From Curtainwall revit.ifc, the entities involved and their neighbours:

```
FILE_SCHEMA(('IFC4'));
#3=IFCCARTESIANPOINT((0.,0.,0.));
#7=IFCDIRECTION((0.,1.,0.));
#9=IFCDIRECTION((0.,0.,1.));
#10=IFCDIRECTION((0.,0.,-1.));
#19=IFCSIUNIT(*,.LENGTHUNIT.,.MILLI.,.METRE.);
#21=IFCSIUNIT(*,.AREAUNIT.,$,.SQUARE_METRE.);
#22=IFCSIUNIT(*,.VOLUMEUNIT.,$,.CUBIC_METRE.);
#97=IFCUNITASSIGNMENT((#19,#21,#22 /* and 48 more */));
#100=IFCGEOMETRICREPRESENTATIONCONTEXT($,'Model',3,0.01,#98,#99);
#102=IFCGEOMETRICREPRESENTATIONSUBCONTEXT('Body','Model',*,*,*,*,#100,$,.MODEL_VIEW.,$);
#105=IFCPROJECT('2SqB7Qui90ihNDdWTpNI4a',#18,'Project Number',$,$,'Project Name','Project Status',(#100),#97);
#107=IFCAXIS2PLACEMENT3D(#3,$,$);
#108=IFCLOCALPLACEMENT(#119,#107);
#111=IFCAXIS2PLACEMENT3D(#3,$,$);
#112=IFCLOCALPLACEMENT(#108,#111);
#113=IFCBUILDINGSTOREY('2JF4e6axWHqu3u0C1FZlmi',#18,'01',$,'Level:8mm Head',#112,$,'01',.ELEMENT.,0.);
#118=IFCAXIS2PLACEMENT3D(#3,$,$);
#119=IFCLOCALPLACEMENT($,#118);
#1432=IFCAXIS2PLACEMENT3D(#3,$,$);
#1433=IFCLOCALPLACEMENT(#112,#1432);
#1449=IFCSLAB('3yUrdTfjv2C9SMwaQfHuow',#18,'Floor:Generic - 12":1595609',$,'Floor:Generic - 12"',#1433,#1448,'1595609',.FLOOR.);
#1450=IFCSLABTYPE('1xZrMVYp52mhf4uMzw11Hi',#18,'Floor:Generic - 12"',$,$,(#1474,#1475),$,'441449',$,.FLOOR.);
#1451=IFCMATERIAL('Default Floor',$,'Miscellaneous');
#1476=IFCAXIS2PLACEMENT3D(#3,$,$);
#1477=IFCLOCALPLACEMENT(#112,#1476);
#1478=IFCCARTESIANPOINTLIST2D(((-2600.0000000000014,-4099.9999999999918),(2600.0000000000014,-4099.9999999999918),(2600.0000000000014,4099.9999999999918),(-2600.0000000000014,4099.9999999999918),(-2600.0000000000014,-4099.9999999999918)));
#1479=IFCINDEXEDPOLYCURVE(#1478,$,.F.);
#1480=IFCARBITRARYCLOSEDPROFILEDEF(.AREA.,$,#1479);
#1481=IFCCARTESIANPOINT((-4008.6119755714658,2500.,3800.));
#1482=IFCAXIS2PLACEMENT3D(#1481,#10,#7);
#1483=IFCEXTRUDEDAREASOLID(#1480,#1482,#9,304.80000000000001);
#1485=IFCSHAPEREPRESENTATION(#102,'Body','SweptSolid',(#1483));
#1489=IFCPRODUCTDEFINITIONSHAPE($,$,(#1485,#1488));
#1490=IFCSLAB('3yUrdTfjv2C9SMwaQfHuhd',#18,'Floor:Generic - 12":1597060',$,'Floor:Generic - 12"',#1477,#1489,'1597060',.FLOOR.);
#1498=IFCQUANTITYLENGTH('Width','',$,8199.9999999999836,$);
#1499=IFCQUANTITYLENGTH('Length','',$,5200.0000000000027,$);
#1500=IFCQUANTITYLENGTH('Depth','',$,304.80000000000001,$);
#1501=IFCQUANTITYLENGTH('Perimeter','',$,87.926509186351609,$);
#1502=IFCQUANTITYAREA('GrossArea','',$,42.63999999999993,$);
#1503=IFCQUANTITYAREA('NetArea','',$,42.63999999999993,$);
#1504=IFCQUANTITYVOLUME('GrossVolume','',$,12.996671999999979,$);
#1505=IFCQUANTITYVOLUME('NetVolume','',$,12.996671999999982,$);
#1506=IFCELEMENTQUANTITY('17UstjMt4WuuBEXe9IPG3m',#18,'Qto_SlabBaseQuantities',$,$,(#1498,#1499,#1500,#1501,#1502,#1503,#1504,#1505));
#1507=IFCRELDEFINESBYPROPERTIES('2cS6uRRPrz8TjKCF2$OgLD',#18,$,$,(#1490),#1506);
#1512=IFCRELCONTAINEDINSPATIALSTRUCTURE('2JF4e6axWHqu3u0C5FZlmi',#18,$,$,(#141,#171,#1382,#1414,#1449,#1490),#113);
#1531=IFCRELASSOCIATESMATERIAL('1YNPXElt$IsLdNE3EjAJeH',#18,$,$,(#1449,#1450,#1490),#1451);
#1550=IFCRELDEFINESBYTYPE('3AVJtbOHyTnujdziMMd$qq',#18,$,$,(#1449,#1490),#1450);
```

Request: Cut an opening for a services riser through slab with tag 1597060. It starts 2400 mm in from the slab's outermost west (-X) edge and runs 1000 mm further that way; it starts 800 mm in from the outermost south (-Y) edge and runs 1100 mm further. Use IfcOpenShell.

```python
import numpy as np
import ifcopenshell
import ifcopenshell.api.feature
import ifcopenshell.api.geometry
import ifcopenshell.api.pset
import ifcopenshell.api.root
import ifcopenshell.geom
import ifcopenshell.util.element
import ifcopenshell.util.placement
import ifcopenshell.util.representation
import ifcopenshell.util.shape
import ifcopenshell.util.unit

model = ifcopenshell.open("Curtainwall revit.ifc")
unit_scale = ifcopenshell.util.unit.calculate_unit_scale(model)
area_scale = ifcopenshell.util.unit.calculate_unit_scale(model, "AREAUNIT")
volume_scale = ifcopenshell.util.unit.calculate_unit_scale(model, "VOLUMEUNIT")
settings = ifcopenshell.geom.settings()


def volume(element):
    """Net volume in cubic metres, openings subtracted."""
    shape = ifcopenshell.geom.create_shape(settings, element)
    return ifcopenshell.util.shape.get_volume(shape.geometry)


slab = model.by_id(1490)
before = volume(slab)

# Extent in the slab's own axes, in metres. The edges named are its -X and -Y sides.
slab_shape = ifcopenshell.geom.create_shape(settings, slab)
vertices = ifcopenshell.util.shape.get_vertices(slab_shape.geometry)
x_min, y_min, bottom = vertices.min(axis=0)
top = vertices[:, 2].max()

opening = ifcopenshell.api.root.create_entity(model, ifc_class="IfcOpeningElement", name="Services riser opening", predefined_type="OPENING")
context = ifcopenshell.util.representation.get_context(model, "Model", "Body", "MODEL_VIEW")
width, depth = 1, 1.1
outline = [(0.0, 0.0), (width, 0.0), (width, depth), (0.0, depth), (0.0, 0.0)]
# Overshoot both faces by 50 mm so the cut is clean.
shape = ifcopenshell.api.geometry.add_slab_representation(
    model, context=context, depth=top - bottom + 0.1, polyline=outline
)
ifcopenshell.api.geometry.assign_representation(model, product=opening, representation=shape)

matrix = ifcopenshell.util.placement.get_local_placement(slab.ObjectPlacement)
matrix[:, 3] = matrix @ np.append(np.array([x_min + 2.4, y_min + 0.8, bottom - 0.05]) / unit_scale, 1.0)
ifcopenshell.api.geometry.edit_object_placement(model, product=opening, matrix=matrix, is_si=False)
ifcopenshell.api.feature.add_feature(model, feature=opening, element=slab)

after = volume(slab)

# Update the slab's stored quantities.
qto = model.by_id(ifcopenshell.util.element.get_pset(slab, "Qto_SlabBaseQuantities", should_inherit=False)["id"])
ifcopenshell.api.pset.edit_qto(model, qto=qto, properties={
    "NetArea": after / (top - bottom) / area_scale,
    "NetVolume": after / volume_scale,
})

print(f"slab volume {before:.3f} -> {after:.3f} m3")

model.write("Curtainwall revit_v2.ifc")
```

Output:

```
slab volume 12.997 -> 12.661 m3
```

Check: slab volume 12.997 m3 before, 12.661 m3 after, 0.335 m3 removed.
